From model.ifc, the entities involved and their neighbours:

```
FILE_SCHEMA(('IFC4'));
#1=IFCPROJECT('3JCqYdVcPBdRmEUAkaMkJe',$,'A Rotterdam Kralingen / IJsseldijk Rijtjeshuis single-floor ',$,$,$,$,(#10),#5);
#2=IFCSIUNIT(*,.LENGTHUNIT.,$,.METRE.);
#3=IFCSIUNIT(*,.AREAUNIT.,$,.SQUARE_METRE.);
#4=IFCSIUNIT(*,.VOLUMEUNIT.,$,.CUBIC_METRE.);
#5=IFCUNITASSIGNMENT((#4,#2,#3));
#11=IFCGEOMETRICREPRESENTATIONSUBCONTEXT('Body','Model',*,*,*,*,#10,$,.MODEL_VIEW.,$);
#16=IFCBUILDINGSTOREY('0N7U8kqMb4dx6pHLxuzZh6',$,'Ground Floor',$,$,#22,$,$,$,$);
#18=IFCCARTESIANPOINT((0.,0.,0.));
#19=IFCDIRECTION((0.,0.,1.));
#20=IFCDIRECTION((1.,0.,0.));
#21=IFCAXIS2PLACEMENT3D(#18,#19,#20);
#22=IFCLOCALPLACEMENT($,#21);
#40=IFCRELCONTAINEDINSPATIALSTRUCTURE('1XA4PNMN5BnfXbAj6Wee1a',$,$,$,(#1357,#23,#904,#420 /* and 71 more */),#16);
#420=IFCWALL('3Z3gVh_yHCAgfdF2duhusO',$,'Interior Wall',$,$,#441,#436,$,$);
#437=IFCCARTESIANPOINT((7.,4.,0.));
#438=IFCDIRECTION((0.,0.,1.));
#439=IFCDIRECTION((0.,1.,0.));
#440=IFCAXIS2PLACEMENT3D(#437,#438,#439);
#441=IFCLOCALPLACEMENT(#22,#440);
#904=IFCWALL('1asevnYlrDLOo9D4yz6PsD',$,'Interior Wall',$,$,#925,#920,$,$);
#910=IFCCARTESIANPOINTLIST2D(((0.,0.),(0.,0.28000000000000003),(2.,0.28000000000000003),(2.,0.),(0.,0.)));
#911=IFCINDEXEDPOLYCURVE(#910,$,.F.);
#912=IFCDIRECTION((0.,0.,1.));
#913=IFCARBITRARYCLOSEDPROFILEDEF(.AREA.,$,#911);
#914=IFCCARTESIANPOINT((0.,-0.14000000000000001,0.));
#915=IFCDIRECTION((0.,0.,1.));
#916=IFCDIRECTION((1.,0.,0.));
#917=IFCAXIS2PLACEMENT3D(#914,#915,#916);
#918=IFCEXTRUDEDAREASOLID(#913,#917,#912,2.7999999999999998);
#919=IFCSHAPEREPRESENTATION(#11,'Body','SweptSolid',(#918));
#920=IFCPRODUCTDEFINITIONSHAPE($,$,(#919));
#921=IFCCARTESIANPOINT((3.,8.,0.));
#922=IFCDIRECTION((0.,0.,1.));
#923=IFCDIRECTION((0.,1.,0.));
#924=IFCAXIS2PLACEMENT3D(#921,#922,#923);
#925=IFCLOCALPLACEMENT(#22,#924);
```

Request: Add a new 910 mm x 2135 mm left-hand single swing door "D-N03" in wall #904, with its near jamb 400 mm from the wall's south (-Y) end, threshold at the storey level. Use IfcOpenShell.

```python
import numpy as np
import ifcopenshell
import ifcopenshell.api.feature
import ifcopenshell.api.geometry
import ifcopenshell.api.root
import ifcopenshell.api.spatial
import ifcopenshell.geom
import ifcopenshell.util.element
import ifcopenshell.util.placement
import ifcopenshell.util.representation
import ifcopenshell.util.shape
import ifcopenshell.util.unit

model = ifcopenshell.open("model.ifc")
unit_scale = ifcopenshell.util.unit.calculate_unit_scale(model)
settings = ifcopenshell.geom.settings()


def volume(element):
    """Net volume in cubic metres, openings subtracted."""
    shape = ifcopenshell.geom.create_shape(settings, element)
    return ifcopenshell.util.shape.get_volume(shape.geometry)


wall = model.by_guid("1asevnYlrDLOo9D4yz6PsD")
storey = ifcopenshell.util.element.get_container(wall, ifc_class="IfcBuildingStorey")
context = ifcopenshell.util.representation.get_context(model, "Model", "Body", "MODEL_VIEW")
before = volume(wall)

width, height, from_end, sill = 0.91, 2.135, 0.4, 0.0  # metres

# The wall runs along its own X axis, and the end named is its -X end.
wall_shape = ifcopenshell.geom.create_shape(settings, wall)
x, y, z = ifcopenshell.util.shape.get_vertices(wall_shape.geometry).T
start = x.min() + from_end
face, thickness = float(y.min()), float(y.max() - y.min())
wall_matrix = ifcopenshell.util.placement.get_local_placement(wall.ObjectPlacement)
level = ifcopenshell.util.placement.get_local_placement(storey.ObjectPlacement)[2, 3]


def in_wall(x, y):
    """Placement at x, y metres in the wall's axes, at sill height."""
    matrix = wall_matrix.copy()
    matrix[:, 3] = wall_matrix @ np.array([x / unit_scale, y / unit_scale, 0.0, 1.0])
    matrix[2, 3] = level + sill / unit_scale
    return matrix


# Opening: a box that overshoots both wall faces by 50 mm.
opening = ifcopenshell.api.root.create_entity(model, ifc_class="IfcOpeningElement", predefined_type="OPENING")
box = ifcopenshell.api.geometry.add_wall_representation(
    model, context=context, length=width, height=height, thickness=thickness + 0.1
)
ifcopenshell.api.geometry.assign_representation(model, product=opening, representation=box)
ifcopenshell.api.geometry.edit_object_placement(model, product=opening, matrix=in_wall(start, face - 0.05), is_si=False)
ifcopenshell.api.feature.add_feature(model, feature=opening, element=wall)

door = ifcopenshell.api.root.create_entity(model, ifc_class="IfcDoor", name="D-N03", predefined_type="DOOR")
door.OverallWidth, door.OverallHeight = width / unit_scale, height / unit_scale
door.OperationType = "SINGLE_SWING_LEFT"
body = ifcopenshell.api.geometry.add_door_representation(
    model,
    context=context,
    overall_width=door.OverallWidth,
    overall_height=door.OverallHeight,
    operation_type="SINGLE_SWING_LEFT",
    lining_properties={"LiningDepth": thickness / unit_scale, "ThresholdDepth": thickness / unit_scale},
)
ifcopenshell.api.geometry.assign_representation(model, product=door, representation=body)
ifcopenshell.api.spatial.assign_container(model, products=[door], relating_structure=storey)
ifcopenshell.api.feature.add_filling(model, opening=opening, element=door)

# The lining spans the wall, so the door starts at the wall face.
ifcopenshell.api.geometry.edit_object_placement(model, product=door, matrix=in_wall(start, face), is_si=False)

after = volume(wall)

print(f"wall volume {before:.3f} -> {after:.3f} m3")

model.write("model_rev.ifc")
```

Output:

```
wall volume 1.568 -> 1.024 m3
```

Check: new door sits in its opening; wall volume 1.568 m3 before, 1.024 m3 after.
